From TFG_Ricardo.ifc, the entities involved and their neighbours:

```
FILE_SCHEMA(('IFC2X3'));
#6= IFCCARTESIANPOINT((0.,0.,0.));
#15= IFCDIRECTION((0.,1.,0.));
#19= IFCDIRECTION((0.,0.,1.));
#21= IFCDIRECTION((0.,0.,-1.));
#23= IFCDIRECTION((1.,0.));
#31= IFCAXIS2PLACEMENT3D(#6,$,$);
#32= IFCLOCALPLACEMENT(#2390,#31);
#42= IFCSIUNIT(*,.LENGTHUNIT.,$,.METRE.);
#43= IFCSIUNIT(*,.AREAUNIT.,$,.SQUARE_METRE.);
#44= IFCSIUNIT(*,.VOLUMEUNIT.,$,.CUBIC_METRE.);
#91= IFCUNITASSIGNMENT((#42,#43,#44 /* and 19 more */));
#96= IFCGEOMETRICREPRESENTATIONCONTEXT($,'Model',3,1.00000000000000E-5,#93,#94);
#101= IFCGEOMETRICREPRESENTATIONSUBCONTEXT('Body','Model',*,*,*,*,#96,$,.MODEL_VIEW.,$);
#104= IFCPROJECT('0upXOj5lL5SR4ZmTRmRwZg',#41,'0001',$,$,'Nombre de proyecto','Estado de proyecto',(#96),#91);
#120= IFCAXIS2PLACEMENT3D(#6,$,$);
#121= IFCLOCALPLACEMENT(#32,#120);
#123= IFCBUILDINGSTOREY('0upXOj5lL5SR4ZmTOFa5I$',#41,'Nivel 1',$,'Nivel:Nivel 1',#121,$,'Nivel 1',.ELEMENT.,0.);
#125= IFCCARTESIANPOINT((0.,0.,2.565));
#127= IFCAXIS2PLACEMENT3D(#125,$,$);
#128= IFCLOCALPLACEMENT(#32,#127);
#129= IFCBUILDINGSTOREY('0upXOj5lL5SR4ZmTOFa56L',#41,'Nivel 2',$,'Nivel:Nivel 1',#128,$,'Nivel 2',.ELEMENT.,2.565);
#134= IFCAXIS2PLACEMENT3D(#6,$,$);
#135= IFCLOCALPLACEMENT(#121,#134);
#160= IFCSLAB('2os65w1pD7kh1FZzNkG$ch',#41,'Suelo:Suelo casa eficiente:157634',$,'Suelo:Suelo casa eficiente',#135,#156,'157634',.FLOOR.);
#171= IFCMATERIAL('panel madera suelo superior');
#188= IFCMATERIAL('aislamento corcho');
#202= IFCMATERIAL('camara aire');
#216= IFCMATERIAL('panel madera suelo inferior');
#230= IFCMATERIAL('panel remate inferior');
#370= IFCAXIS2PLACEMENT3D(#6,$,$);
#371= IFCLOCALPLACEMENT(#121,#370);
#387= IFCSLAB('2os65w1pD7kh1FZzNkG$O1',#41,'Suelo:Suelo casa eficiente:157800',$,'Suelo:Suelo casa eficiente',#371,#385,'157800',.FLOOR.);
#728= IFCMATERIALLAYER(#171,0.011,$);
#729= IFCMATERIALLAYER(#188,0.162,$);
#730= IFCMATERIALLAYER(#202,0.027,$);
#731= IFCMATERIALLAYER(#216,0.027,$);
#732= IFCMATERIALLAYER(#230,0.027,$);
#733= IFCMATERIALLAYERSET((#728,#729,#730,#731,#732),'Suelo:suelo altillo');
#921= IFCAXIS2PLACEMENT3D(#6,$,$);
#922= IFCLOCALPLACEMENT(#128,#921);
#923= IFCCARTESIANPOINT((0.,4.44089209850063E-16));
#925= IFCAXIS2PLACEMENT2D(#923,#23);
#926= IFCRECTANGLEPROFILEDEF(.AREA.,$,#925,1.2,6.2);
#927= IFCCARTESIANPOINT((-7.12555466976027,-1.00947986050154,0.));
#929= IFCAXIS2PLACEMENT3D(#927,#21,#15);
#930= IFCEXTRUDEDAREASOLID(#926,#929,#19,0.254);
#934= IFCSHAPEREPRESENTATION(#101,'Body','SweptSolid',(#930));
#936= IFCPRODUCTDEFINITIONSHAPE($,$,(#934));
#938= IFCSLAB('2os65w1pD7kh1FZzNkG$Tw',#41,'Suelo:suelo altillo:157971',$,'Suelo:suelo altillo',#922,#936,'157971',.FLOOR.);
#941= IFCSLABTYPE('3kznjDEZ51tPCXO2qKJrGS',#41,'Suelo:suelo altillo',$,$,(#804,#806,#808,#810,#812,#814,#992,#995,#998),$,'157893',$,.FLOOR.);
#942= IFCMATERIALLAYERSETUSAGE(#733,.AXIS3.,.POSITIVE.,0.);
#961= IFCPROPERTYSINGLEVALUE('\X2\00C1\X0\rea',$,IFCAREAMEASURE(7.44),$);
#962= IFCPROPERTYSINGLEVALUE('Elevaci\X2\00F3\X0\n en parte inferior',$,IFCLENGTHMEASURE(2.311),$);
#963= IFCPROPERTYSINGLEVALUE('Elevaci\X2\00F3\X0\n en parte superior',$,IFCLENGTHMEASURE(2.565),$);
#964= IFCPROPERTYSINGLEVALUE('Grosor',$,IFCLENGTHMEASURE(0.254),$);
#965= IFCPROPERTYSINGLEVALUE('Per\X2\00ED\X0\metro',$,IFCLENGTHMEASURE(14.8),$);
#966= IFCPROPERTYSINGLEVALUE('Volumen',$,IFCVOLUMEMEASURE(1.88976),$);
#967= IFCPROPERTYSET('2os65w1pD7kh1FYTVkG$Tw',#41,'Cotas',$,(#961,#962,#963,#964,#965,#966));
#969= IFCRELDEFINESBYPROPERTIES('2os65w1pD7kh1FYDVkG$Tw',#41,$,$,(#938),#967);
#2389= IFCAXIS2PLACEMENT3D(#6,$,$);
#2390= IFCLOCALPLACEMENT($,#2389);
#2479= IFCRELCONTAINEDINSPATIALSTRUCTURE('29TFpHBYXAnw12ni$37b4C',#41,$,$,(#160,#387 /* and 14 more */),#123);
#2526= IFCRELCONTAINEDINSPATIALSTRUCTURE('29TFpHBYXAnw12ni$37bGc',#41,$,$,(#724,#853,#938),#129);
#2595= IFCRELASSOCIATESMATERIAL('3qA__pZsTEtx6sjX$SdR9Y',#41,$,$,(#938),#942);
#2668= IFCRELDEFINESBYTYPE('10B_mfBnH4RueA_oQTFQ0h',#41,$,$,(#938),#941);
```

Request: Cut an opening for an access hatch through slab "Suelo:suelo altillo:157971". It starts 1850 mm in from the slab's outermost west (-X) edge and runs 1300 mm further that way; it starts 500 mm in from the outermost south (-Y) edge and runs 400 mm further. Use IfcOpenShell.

```python
import numpy as np
import ifcopenshell
import ifcopenshell.api.feature
import ifcopenshell.api.geometry
import ifcopenshell.api.pset
import ifcopenshell.api.root
import ifcopenshell.geom
import ifcopenshell.util.element
import ifcopenshell.util.placement
import ifcopenshell.util.representation
import ifcopenshell.util.shape
import ifcopenshell.util.unit

model = ifcopenshell.open("TFG_Ricardo.ifc")
unit_scale = ifcopenshell.util.unit.calculate_unit_scale(model)
area_scale = ifcopenshell.util.unit.calculate_unit_scale(model, "AREAUNIT")
volume_scale = ifcopenshell.util.unit.calculate_unit_scale(model, "VOLUMEUNIT")
settings = ifcopenshell.geom.settings()


def volume(element):
    """Net volume in cubic metres, openings subtracted."""
    shape = ifcopenshell.geom.create_shape(settings, element)
    return ifcopenshell.util.shape.get_volume(shape.geometry)


slab = model.by_id(938)
before = volume(slab)

# Extent in the slab's own axes, in metres. The edges named are its -X and -Y sides.
slab_shape = ifcopenshell.geom.create_shape(settings, slab)
vertices = ifcopenshell.util.shape.get_vertices(slab_shape.geometry)
x_min, y_min, bottom = vertices.min(axis=0)
top = vertices[:, 2].max()

opening = ifcopenshell.api.root.create_entity(model, ifc_class="IfcOpeningElement", name="Access hatch opening")
context = ifcopenshell.util.representation.get_context(model, "Model", "Body", "MODEL_VIEW")
width, depth = 1.3, 0.4
outline = [(0.0, 0.0), (width, 0.0), (width, depth), (0.0, depth), (0.0, 0.0)]
# Overshoot both faces by 50 mm so the cut is clean.
shape = ifcopenshell.api.geometry.add_slab_representation(
    model, context=context, depth=top - bottom + 0.1, polyline=outline
)
ifcopenshell.api.geometry.assign_representation(model, product=opening, representation=shape)

matrix = ifcopenshell.util.placement.get_local_placement(slab.ObjectPlacement)
matrix[:, 3] = matrix @ np.append(np.array([x_min + 1.85, y_min + 0.5, bottom - 0.05]) / unit_scale, 1.0)
ifcopenshell.api.geometry.edit_object_placement(model, product=opening, matrix=matrix, is_si=False)
ifcopenshell.api.feature.add_feature(model, feature=opening, element=slab)

after = volume(slab)

# Update the slab's stored quantities.
pset = model.by_id(ifcopenshell.util.element.get_pset(slab, "Cotas", should_inherit=False)["id"])
ifcopenshell.api.pset.edit_pset(model, pset=pset, properties={
    "Área": model.create_entity("IfcAreaMeasure", after / (top - bottom) / area_scale),
    "Volumen": model.create_entity("IfcVolumeMeasure", after / volume_scale),
})

print(f"slab volume {before:.3f} -> {after:.3f} m3")

model.write("TFG_Ricardo_rev.ifc")
```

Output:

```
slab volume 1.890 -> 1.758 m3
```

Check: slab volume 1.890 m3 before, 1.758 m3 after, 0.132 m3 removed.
